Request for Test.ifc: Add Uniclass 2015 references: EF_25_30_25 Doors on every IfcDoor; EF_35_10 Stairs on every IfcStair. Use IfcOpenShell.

First a look at what the model holds.

```python
import ifcopenshell

model = ifcopenshell.open("Test.ifc")
print(model.schema)
print("classifications:", [c.Name for c in model.by_type("IfcClassification")])
for ifc_class in ("IfcDoor", "IfcRoof", "IfcStair", "IfcWall", "IfcWindow"):
    print(ifc_class, len(model.by_type(ifc_class)))
```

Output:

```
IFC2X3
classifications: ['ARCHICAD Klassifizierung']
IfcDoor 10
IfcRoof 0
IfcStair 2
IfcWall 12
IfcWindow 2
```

```python
import ifcopenshell
import ifcopenshell.api.classification

model = ifcopenshell.open("Test.ifc")

# IFC2X3 requires Source and Edition and has no link from the project to the system.
system = model.create_entity("IfcClassification", Source="NBS", Edition="2015", Name="Uniclass 2015")

codes = {
    "IfcDoor": ("EF_25_30_25", "Doors"),
    "IfcStair": ("EF_35_10", "Stairs"),
}
for ifc_class, (code, name) in codes.items():
    products = model.by_type(ifc_class)
    ifcopenshell.api.classification.add_reference(
        model, products=products, classification=system, identification=code, name=name
    )
    print(code, len(products))

model.write("Test_rev.ifc")
```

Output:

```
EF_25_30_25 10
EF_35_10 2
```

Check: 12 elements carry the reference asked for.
